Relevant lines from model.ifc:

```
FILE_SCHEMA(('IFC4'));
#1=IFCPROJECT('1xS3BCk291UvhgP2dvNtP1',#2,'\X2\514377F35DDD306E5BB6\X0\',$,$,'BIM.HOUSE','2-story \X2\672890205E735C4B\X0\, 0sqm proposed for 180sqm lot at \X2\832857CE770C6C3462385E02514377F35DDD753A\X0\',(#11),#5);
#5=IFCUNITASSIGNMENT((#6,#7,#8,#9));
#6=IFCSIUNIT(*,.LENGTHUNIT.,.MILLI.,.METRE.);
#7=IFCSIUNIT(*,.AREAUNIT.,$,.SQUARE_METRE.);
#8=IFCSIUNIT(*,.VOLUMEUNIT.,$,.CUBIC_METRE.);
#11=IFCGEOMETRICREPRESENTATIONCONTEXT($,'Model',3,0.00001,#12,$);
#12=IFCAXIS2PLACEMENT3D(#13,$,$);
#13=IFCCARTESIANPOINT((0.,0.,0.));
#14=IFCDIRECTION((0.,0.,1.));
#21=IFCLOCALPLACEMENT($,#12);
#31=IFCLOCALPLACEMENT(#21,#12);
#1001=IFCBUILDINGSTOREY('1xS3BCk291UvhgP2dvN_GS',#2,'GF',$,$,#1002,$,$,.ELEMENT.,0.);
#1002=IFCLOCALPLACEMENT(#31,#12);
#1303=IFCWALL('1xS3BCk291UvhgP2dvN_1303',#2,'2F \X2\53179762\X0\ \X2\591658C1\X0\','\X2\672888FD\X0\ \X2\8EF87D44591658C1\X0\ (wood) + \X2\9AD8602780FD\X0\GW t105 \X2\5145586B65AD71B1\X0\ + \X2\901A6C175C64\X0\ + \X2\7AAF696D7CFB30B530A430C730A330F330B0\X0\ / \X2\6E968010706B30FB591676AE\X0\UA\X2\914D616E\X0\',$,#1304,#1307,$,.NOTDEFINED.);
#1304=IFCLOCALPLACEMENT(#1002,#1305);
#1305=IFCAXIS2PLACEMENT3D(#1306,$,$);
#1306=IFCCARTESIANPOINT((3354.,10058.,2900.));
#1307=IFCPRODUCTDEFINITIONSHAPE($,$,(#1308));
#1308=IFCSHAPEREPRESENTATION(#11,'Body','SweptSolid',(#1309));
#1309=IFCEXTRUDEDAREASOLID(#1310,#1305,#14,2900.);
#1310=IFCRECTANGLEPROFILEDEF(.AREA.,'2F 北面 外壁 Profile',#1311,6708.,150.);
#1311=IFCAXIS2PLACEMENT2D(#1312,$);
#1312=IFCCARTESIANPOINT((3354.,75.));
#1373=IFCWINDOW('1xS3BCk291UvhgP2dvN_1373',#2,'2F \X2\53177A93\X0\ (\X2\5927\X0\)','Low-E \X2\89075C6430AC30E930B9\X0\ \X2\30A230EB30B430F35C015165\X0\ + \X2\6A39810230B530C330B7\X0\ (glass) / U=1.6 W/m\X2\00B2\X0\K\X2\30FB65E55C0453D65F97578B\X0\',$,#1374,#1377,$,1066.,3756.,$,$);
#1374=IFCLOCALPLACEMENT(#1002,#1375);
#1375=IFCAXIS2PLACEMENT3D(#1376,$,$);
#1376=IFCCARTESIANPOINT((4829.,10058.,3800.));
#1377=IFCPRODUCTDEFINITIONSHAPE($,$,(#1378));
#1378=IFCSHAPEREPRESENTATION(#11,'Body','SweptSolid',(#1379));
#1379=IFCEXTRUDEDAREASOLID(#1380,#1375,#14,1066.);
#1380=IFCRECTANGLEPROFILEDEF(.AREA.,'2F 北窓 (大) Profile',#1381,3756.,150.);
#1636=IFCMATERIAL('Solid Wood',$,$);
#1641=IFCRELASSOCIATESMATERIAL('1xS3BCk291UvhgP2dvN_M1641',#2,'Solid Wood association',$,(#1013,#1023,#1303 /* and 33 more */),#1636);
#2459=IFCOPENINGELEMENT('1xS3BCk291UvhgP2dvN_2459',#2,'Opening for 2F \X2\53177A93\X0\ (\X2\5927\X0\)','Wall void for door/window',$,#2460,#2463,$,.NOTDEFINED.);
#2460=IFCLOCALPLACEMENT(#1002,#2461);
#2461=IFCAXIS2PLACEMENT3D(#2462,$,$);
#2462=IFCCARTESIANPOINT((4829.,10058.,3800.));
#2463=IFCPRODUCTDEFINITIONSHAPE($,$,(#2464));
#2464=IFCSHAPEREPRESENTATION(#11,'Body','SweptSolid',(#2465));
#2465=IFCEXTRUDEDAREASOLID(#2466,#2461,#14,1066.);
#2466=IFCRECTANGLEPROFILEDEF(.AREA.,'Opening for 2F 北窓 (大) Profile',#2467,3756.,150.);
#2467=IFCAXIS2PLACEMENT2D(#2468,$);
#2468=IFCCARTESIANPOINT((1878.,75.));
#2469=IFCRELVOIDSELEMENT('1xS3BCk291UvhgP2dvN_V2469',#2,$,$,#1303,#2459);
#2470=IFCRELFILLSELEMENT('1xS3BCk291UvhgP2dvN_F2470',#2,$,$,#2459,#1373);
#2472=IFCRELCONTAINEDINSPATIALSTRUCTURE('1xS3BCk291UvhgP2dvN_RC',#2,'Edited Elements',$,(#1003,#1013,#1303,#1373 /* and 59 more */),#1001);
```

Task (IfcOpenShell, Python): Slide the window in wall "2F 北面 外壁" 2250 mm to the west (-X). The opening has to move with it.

```python
import ifcopenshell
import ifcopenshell.api.geometry
import ifcopenshell.util.placement

model = ifcopenshell.open("model.ifc")

window = model.by_guid("1xS3BCk291UvhgP2dvN_1373")
opening = window.FillsVoids[0].RelatingOpeningElement
wall = opening.VoidsElements[0].RelatingBuildingElement

wall_matrix = ifcopenshell.util.placement.get_local_placement(wall.ObjectPlacement)
shift = wall_matrix[:3, 0] * -2250.0
before = ifcopenshell.util.placement.get_local_placement(window.ObjectPlacement)[:3, 3].copy()

# The window is not placed relative to its opening, so move both.
for product in (opening, window):
    matrix = ifcopenshell.util.placement.get_local_placement(product.ObjectPlacement)
    matrix[:3, 3] += shift
    ifcopenshell.api.geometry.edit_object_placement(model, product=product, matrix=matrix, is_si=False)

after = ifcopenshell.util.placement.get_local_placement(window.ObjectPlacement)[:3, 3]
print("window moved by", (after - before).round(3) + 0.0)

model.write("model_rev.ifc")
```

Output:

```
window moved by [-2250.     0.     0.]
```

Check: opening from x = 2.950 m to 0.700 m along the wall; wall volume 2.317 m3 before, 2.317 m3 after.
